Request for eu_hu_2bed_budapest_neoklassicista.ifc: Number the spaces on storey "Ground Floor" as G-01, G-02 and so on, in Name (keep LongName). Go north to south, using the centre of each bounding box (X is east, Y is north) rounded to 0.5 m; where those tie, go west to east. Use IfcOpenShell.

First a look at what the model holds.

```python
import ifcopenshell
import ifcopenshell.util.element
import ifcopenshell.util.placement

model = ifcopenshell.open("eu_hu_2bed_budapest_neoklassicista.ifc")
print(model.schema)
storey = next(s for s in model.by_type("IfcBuildingStorey") if s.Name == "Ground Floor")
spaces = [e for e in ifcopenshell.util.element.get_decomposition(storey) if e.is_a("IfcSpace")]
for e in sorted(spaces, key=lambda e: e.id()):
    origin = ifcopenshell.util.placement.get_local_placement(e.ObjectPlacement)[:3, 3]
    print(e.id(), e.Name, e.LongName, origin.round(2) + 0.0, sep=" | ")
```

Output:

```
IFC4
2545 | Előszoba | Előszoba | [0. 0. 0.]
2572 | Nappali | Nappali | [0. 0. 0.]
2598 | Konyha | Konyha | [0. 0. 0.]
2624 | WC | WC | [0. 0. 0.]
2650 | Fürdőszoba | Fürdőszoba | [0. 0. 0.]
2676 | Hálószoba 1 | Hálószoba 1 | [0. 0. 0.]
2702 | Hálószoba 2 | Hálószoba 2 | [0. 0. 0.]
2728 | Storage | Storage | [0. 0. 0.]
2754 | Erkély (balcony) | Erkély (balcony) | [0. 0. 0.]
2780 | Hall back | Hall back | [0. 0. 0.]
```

```python
import ifcopenshell
import ifcopenshell.geom
import ifcopenshell.util.element
import ifcopenshell.util.shape

model = ifcopenshell.open("eu_hu_2bed_budapest_neoklassicista.ifc")
settings = ifcopenshell.geom.settings()
settings.set("use-world-coords", True)


def centre(element):
    shape = ifcopenshell.geom.create_shape(settings, element)
    return ifcopenshell.util.shape.get_bbox_centroid(shape.geometry)


storey = next(s for s in model.by_type("IfcBuildingStorey") if s.Name == "Ground Floor")
spaces = [e for e in ifcopenshell.util.element.get_decomposition(storey) if e.is_a("IfcSpace")]

# Insertion points can sit at a corner or the storey origin, so sort by the geometry (in metres).
centres = {e: centre(e) for e in spaces}
spaces.sort(key=lambda e: (-round(centres[e][1] / 0.5), centres[e][0]))

for i, e in enumerate(spaces, start=1):
    number = f"G-{i:02d}"
    e.Name = number
    print(e.id(), number)

model.write("eu_hu_2bed_budapest_neoklassicista_v2.ifc")
```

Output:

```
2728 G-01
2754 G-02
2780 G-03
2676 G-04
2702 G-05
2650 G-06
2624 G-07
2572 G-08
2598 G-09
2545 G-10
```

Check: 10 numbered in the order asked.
